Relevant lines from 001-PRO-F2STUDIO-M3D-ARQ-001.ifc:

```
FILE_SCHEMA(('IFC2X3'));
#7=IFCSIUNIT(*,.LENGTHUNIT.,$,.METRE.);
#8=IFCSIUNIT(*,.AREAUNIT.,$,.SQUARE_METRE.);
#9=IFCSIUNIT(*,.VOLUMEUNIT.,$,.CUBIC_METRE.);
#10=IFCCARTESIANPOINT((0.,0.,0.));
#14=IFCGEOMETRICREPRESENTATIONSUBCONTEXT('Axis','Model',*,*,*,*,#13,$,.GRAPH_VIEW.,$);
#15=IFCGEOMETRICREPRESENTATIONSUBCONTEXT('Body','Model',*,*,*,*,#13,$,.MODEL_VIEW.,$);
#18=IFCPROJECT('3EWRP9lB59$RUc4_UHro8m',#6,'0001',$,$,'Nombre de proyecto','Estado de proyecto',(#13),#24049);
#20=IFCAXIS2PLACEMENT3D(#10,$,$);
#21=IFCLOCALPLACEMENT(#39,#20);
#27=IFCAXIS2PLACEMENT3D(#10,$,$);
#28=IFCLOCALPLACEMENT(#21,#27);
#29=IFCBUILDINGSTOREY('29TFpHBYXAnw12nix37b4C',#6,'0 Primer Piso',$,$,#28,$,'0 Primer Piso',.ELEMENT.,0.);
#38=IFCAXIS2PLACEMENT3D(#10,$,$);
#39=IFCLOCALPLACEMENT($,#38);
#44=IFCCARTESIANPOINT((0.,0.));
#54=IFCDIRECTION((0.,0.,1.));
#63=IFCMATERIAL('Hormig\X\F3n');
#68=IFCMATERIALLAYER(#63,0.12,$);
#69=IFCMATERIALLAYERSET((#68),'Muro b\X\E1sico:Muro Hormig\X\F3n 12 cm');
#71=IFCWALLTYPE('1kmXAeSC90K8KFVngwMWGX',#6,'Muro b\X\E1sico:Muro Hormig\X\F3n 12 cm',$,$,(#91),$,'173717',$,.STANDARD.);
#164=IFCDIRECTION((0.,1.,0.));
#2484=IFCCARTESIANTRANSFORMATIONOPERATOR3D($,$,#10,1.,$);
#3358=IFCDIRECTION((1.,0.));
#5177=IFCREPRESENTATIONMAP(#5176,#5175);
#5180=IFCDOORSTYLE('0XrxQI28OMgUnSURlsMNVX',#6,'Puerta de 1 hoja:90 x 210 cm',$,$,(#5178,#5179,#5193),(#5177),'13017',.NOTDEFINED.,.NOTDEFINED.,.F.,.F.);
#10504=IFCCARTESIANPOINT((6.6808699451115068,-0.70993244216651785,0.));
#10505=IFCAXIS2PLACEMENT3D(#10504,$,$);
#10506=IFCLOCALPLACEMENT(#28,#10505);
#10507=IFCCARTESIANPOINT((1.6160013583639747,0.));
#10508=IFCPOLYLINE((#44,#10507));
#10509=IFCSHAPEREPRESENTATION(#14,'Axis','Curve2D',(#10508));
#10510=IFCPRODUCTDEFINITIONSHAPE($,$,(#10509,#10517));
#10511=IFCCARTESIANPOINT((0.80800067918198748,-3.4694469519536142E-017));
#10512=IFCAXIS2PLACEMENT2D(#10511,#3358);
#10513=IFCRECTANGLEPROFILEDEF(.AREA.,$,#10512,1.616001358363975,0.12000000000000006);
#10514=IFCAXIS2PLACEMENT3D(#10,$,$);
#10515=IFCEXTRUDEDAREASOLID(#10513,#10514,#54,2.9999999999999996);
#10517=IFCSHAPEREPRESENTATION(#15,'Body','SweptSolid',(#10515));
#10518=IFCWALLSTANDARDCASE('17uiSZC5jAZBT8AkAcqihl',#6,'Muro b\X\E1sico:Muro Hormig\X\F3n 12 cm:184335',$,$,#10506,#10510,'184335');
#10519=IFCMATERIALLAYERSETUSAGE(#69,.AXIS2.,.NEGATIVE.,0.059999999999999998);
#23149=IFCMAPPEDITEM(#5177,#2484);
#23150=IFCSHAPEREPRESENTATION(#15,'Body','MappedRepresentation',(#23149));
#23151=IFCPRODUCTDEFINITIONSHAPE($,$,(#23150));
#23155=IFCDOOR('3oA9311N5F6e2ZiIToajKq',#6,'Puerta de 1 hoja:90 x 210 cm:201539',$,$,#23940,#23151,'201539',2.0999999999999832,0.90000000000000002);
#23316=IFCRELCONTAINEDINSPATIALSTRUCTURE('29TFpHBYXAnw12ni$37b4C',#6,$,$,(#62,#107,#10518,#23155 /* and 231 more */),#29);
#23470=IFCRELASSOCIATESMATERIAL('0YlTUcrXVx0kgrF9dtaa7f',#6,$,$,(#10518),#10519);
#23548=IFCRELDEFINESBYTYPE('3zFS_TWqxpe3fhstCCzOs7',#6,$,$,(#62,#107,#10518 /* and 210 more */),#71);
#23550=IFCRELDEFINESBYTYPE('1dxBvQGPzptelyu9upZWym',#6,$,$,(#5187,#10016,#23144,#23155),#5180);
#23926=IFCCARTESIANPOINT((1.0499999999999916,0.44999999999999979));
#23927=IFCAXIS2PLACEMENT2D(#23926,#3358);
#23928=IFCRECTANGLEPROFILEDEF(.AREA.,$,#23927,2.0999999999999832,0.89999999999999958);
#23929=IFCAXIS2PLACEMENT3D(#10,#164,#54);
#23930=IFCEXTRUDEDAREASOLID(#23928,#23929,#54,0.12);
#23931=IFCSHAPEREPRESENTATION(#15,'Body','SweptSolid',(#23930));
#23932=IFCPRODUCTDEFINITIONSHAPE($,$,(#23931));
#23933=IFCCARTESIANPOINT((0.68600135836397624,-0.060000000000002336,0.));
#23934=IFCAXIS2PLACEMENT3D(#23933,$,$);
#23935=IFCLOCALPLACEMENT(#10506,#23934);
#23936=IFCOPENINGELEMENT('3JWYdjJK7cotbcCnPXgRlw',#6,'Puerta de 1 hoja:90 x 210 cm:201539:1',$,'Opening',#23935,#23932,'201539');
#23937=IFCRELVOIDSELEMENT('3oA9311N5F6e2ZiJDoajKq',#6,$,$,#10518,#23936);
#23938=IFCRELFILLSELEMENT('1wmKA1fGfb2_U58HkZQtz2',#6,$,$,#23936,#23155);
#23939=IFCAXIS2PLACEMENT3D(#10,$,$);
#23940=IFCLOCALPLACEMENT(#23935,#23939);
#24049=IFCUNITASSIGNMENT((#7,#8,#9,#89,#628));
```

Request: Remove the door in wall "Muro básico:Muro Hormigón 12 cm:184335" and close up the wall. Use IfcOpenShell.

```python
import ifcopenshell
import ifcopenshell.api.feature
import ifcopenshell.api.root
import ifcopenshell.geom
import ifcopenshell.util.shape

model = ifcopenshell.open("001-PRO-F2STUDIO-M3D-ARQ-001.ifc")
settings = ifcopenshell.geom.settings()


def volume(element):
    """Net volume in cubic metres, openings subtracted."""
    shape = ifcopenshell.geom.create_shape(settings, element)
    return ifcopenshell.util.shape.get_volume(shape.geometry)


door = model.by_guid("3oA9311N5F6e2ZiIToajKq")
opening = door.FillsVoids[0].RelatingOpeningElement
wall = opening.VoidsElements[0].RelatingBuildingElement
before = volume(wall)

ifcopenshell.api.root.remove_product(model, product=door)
ifcopenshell.api.feature.remove_feature(model, feature=opening)

after = volume(wall)

print(f"wall volume {before:.3f} -> {after:.3f} m3")

model.write("001-PRO-F2STUDIO-M3D-ARQ-001_edited.ifc")
```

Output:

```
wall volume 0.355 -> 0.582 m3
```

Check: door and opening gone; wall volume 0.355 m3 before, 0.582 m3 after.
